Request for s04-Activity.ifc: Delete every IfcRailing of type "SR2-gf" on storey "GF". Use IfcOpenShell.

First a look at what the model holds.

```python
import ifcopenshell
import ifcopenshell.util.element

model = ifcopenshell.open("s04-Activity.ifc")
print(model.schema)
storey = next(s for s in model.by_type("IfcBuildingStorey") if s.Name == "GF")
railings = [e for e in ifcopenshell.util.element.get_decomposition(storey) if e.is_a("IfcRailing")]
seen = {}
for e in railings:
    element_type = ifcopenshell.util.element.get_type(e)
    name = element_type.Name if element_type not in (None, e) else None
    seen[name] = seen.get(name, 0) + 1
for name, count in sorted(seen.items(), key=str):
    print(count, "x", name)
```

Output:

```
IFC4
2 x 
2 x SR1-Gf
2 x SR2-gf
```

```python
import ifcopenshell
import ifcopenshell.api.root
import ifcopenshell.util.element

model = ifcopenshell.open("s04-Activity.ifc")

storey = next(s for s in model.by_type("IfcBuildingStorey") if s.Name == "GF")
railings = [e for e in ifcopenshell.util.element.get_decomposition(storey) if e.is_a("IfcRailing")]
targets = [e for e in railings if (t := ifcopenshell.util.element.get_type(e)) not in (None, e) and t.Name == "SR2-gf"]

for e in targets:
    ifcopenshell.api.root.remove_product(model, product=e)
print(len(targets), "removed")

model.write("s04-Activity_rev.ifc")
```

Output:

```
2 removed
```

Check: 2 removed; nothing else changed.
